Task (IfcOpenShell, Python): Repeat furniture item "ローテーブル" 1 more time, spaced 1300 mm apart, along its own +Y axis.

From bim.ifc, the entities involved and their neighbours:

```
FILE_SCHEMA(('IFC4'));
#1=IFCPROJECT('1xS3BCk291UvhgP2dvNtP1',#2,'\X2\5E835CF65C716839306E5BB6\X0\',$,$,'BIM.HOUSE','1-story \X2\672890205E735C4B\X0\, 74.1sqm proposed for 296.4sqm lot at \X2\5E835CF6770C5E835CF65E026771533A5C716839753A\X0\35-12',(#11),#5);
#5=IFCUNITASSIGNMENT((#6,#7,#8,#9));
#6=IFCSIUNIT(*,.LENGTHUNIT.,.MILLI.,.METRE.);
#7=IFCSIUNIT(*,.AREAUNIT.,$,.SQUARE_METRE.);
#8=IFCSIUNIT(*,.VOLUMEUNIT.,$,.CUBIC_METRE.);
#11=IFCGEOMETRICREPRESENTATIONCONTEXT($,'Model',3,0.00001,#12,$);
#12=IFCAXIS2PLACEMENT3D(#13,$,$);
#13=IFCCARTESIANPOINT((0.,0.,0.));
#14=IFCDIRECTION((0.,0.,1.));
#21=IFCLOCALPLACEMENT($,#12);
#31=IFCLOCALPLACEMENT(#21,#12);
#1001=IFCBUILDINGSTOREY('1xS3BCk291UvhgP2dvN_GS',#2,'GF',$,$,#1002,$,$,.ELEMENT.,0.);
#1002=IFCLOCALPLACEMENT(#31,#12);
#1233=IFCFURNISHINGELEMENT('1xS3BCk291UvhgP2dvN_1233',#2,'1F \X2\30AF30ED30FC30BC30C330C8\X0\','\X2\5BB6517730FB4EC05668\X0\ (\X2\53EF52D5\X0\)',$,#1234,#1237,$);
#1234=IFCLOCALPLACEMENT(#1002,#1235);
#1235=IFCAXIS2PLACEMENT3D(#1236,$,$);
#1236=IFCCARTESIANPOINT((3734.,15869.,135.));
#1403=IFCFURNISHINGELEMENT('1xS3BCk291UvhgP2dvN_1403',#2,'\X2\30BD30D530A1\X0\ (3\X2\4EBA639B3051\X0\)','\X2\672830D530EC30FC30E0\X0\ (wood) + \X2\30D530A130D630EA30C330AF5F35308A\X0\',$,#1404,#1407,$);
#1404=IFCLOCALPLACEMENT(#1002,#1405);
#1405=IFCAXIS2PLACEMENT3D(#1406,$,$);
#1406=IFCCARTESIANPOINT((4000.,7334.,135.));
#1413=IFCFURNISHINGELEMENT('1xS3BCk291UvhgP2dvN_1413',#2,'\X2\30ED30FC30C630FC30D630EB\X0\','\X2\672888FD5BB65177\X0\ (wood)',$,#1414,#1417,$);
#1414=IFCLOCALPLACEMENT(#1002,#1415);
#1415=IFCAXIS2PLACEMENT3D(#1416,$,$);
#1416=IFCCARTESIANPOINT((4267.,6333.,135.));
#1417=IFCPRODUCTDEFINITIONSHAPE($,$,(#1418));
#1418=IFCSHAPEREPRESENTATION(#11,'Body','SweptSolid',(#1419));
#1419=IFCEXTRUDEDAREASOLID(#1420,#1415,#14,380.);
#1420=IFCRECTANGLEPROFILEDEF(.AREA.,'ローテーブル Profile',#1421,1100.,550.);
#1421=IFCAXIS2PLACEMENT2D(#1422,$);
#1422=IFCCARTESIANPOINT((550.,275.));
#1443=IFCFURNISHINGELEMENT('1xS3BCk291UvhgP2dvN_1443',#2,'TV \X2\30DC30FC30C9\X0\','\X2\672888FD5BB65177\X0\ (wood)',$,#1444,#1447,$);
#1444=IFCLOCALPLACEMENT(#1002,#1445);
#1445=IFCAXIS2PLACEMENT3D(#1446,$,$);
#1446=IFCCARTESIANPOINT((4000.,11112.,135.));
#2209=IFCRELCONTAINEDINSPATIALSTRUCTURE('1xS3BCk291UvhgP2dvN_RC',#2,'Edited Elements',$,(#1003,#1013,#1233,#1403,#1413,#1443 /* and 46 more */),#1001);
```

```python
import ifcopenshell
import ifcopenshell.api.geometry
import ifcopenshell.api.root
import ifcopenshell.util.element
import ifcopenshell.util.placement
import ifcopenshell.util.unit

model = ifcopenshell.open("bim.ifc")
unit_scale = ifcopenshell.util.unit.calculate_unit_scale(model)


def reuse_history(source, copy):
    """copy_class also copies each property set's owner history, people and application; keep the originals."""
    for rel in copy.IsDefinedBy:
        if rel.is_a("IfcRelDefinesByProperties") and (history := rel.RelatingPropertyDefinition.OwnerHistory):
            rel.RelatingPropertyDefinition.OwnerHistory = source.OwnerHistory
            ifcopenshell.util.element.remove_deep2(model, history)


source = model.by_id(1413)
base = ifcopenshell.util.placement.get_local_placement(source.ObjectPlacement)
step = base[:3, 1] * 1.3 / unit_scale

for i in range(1, 2):
    copy = ifcopenshell.api.root.copy_class(model, product=source)
    copy.Representation = ifcopenshell.util.element.copy_deep(
        model, source.Representation, exclude=["IfcGeometricRepresentationContext", "IfcRepresentationMap"]
    )
    reuse_history(source, copy)
    matrix = base.copy()
    matrix[:3, 3] += i * step
    print("added at", matrix[:3, 3].round(3) + 0.0)
    ifcopenshell.api.geometry.edit_object_placement(model, product=copy, matrix=matrix, is_si=False)

model.write("bim-out.ifc")
```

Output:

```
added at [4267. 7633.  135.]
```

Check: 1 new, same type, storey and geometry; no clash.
